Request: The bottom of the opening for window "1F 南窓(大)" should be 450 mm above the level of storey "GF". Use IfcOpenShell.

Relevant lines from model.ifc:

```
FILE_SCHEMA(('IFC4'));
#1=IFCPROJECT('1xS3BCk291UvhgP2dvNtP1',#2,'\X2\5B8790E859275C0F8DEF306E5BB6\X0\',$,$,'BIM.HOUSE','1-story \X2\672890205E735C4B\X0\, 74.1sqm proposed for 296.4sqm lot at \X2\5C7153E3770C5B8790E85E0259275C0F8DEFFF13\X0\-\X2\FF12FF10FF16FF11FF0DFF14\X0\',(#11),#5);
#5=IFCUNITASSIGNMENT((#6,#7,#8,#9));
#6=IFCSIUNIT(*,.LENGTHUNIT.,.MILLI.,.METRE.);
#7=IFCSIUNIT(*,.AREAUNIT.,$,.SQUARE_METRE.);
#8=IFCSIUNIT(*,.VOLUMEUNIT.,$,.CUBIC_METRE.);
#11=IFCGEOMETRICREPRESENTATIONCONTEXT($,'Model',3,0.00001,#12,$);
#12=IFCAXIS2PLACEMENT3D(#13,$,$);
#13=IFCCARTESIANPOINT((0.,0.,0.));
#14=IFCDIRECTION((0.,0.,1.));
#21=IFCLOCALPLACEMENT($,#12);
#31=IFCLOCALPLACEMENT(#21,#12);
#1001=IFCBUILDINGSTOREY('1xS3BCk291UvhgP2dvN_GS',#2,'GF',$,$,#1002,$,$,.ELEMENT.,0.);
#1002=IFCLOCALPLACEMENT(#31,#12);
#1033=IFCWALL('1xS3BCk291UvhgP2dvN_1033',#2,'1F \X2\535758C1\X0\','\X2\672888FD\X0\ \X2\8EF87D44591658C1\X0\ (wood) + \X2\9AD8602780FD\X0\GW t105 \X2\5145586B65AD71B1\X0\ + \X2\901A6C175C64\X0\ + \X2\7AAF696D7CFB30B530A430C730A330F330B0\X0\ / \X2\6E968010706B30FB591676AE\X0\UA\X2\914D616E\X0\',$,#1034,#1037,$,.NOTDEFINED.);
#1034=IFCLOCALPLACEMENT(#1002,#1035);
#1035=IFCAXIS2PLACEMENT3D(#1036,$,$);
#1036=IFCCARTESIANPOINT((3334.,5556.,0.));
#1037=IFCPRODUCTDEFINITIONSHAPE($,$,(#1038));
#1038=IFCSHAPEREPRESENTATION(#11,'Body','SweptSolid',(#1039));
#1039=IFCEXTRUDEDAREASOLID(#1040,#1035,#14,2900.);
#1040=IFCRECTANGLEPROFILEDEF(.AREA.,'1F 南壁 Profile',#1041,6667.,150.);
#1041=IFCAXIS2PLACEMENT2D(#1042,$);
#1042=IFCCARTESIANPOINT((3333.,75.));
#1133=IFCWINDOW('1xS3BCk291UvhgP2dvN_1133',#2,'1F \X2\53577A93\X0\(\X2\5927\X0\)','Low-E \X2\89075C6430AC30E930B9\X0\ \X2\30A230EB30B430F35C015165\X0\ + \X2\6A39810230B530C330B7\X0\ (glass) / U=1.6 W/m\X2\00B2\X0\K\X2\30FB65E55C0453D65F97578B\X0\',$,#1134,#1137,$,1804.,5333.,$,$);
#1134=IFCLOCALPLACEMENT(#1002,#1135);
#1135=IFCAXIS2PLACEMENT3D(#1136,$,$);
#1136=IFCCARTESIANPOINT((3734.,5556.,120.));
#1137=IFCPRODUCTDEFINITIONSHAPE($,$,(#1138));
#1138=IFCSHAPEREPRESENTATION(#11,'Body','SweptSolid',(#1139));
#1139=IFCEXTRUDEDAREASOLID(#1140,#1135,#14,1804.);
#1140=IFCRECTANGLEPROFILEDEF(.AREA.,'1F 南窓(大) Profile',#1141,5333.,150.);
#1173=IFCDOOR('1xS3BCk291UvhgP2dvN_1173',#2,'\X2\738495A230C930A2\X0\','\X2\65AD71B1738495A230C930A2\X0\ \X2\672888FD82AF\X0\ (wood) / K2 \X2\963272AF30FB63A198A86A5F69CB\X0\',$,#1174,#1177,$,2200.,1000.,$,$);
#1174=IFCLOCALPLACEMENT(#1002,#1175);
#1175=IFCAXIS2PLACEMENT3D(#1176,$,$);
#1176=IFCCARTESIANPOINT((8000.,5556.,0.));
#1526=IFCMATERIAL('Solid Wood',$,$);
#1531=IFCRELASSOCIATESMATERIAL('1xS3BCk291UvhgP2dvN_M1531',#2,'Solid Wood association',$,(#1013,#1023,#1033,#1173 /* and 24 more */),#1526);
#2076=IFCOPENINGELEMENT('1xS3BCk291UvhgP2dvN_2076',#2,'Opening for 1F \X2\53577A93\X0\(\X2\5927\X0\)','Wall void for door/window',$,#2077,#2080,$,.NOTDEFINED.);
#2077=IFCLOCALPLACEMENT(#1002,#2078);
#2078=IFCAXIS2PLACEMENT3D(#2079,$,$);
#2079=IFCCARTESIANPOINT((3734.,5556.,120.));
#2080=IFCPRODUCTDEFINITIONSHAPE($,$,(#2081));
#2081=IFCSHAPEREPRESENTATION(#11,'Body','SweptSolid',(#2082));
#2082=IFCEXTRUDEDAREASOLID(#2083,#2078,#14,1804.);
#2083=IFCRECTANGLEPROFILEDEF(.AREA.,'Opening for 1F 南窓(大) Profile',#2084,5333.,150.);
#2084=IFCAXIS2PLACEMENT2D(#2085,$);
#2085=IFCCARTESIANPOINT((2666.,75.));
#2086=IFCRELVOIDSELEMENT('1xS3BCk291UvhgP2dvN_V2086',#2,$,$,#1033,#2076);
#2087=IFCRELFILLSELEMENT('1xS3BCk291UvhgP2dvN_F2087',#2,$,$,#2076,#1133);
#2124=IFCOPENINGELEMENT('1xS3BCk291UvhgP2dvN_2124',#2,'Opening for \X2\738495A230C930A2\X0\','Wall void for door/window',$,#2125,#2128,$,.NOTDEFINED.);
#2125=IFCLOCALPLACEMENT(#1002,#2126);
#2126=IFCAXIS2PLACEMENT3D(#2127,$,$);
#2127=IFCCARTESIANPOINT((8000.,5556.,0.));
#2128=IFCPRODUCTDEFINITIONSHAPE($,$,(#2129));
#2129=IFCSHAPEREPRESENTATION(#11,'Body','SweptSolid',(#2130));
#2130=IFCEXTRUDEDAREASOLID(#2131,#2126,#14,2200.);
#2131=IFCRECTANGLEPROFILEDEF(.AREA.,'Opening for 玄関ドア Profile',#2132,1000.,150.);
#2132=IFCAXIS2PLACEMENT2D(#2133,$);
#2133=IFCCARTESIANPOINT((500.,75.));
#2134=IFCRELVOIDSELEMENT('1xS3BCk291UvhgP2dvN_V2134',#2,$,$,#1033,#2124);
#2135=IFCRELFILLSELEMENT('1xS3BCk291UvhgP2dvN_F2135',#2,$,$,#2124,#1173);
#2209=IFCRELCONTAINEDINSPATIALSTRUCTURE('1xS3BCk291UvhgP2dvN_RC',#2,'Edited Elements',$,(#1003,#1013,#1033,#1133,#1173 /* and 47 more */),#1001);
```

```python
import numpy as np
import ifcopenshell
import ifcopenshell.api.geometry
import ifcopenshell.geom
import ifcopenshell.util.element
import ifcopenshell.util.placement
import ifcopenshell.util.shape
import ifcopenshell.util.unit

model = ifcopenshell.open("model.ifc")
unit_scale = ifcopenshell.util.unit.calculate_unit_scale(model)

window = model.by_guid("1xS3BCk291UvhgP2dvN_1133")
opening = window.FillsVoids[0].RelatingOpeningElement
storey = ifcopenshell.util.element.get_container(window, ifc_class="IfcBuildingStorey")
level = ifcopenshell.util.placement.get_local_placement(storey.ObjectPlacement)[2, 3]

# The opening's origin need not be at the sill, so measure its lowest point.
shape = ifcopenshell.geom.create_shape(ifcopenshell.geom.settings(), opening)
bottom = ifcopenshell.util.shape.get_shape_bottom_elevation(shape, shape.geometry) / unit_scale
dz = level + 0.45 / unit_scale - bottom

shift = np.array([0.0, 0.0, dz])
# The window is not placed relative to its opening, so move both.
for product in (opening, window):
    matrix = ifcopenshell.util.placement.get_local_placement(product.ObjectPlacement)
    matrix[:3, 3] += shift
    ifcopenshell.api.geometry.edit_object_placement(model, product=product, matrix=matrix, is_si=False)

print(f"moved by {dz * unit_scale:+.3f} m")

model.write("model_rev.ifc")
```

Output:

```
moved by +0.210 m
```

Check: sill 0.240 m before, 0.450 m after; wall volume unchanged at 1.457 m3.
